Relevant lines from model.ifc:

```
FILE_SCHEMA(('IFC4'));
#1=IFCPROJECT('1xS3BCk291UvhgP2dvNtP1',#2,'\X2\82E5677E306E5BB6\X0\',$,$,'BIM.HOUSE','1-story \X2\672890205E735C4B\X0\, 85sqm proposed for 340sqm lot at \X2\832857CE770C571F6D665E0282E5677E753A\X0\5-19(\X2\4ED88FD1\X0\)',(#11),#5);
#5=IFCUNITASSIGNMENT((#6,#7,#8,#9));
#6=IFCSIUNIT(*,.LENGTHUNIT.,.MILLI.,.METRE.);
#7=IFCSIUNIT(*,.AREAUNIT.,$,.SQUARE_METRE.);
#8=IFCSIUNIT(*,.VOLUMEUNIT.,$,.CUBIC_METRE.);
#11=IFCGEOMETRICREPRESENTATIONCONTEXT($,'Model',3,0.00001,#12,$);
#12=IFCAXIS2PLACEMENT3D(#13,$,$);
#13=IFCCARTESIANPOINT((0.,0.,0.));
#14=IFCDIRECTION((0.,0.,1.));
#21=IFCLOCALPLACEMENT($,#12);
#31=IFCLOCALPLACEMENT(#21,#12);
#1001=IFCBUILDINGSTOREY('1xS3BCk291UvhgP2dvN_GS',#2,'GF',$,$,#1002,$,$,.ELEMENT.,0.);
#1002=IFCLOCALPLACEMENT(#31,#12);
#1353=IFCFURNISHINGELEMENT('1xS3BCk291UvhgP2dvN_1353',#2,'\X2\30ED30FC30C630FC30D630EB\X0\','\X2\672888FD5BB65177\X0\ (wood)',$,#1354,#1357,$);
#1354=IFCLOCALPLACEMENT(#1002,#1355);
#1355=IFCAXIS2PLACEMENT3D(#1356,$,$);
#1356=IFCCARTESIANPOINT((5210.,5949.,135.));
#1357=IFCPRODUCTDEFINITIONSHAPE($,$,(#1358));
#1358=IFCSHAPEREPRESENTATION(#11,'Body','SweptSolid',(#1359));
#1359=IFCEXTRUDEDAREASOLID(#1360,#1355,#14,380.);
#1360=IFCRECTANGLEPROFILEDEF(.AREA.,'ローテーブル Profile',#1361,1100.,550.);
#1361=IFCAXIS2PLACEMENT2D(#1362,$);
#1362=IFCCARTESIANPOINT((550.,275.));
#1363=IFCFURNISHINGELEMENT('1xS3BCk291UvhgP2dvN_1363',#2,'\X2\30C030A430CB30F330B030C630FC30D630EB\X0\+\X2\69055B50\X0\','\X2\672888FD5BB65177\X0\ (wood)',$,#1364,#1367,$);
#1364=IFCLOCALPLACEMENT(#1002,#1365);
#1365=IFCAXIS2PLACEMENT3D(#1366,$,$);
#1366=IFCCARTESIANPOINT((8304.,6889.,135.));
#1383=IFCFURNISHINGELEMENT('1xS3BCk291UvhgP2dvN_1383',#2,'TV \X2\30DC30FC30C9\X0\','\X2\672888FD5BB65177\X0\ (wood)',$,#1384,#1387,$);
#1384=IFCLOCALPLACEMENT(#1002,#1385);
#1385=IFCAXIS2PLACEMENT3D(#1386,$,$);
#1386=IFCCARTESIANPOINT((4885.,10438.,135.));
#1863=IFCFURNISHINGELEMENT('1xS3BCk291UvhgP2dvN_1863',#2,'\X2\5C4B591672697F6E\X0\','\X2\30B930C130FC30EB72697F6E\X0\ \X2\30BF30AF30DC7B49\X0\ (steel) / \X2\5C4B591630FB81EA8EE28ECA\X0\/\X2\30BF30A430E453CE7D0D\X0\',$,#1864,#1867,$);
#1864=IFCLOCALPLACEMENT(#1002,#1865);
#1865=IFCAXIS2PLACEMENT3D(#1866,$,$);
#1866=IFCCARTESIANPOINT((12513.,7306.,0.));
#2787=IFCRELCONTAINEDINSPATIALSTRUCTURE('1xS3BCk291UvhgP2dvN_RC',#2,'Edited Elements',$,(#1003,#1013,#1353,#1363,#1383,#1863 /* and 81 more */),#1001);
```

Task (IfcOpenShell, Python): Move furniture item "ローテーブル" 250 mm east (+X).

```python
import ifcopenshell
import ifcopenshell.api.geometry
import ifcopenshell.util.placement

model = ifcopenshell.open("model.ifc")

item = model.by_guid("1xS3BCk291UvhgP2dvN_1353")
matrix = ifcopenshell.util.placement.get_local_placement(item.ObjectPlacement)
matrix[0, 3] += 250.0
ifcopenshell.api.geometry.edit_object_placement(model, product=item, matrix=matrix, is_si=False)

print(ifcopenshell.util.placement.get_local_placement(item.ObjectPlacement).round(3) + 0.0)

model.write("model_updated.ifc")
```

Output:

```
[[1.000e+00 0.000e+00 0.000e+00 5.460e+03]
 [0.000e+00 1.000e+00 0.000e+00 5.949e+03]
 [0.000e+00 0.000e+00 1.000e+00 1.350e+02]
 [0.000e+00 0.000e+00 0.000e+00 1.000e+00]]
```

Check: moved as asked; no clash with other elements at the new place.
